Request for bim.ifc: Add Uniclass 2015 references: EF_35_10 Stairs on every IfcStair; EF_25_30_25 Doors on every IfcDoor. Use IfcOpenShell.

First a look at what the model holds.

```python
import ifcopenshell

model = ifcopenshell.open("bim.ifc")
print(model.schema)
print("classifications:", [c.Name for c in model.by_type("IfcClassification")])
for ifc_class in ("IfcDoor", "IfcRoof", "IfcStair", "IfcWall", "IfcWindow"):
    print(ifc_class, len(model.by_type(ifc_class)))
```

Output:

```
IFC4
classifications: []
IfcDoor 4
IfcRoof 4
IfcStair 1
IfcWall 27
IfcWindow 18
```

```python
import ifcopenshell
import ifcopenshell.api.classification

model = ifcopenshell.open("bim.ifc")

system = ifcopenshell.api.classification.add_classification(model, classification="Uniclass 2015")

codes = {
    "IfcStair": ("EF_35_10", "Stairs"),
    "IfcDoor": ("EF_25_30_25", "Doors"),
}
for ifc_class, (code, name) in codes.items():
    products = model.by_type(ifc_class)
    ifcopenshell.api.classification.add_reference(
        model, products=products, classification=system, identification=code, name=name
    )
    print(code, len(products))

model.write("bim-out.ifc")
```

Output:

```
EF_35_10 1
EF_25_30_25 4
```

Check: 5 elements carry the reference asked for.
